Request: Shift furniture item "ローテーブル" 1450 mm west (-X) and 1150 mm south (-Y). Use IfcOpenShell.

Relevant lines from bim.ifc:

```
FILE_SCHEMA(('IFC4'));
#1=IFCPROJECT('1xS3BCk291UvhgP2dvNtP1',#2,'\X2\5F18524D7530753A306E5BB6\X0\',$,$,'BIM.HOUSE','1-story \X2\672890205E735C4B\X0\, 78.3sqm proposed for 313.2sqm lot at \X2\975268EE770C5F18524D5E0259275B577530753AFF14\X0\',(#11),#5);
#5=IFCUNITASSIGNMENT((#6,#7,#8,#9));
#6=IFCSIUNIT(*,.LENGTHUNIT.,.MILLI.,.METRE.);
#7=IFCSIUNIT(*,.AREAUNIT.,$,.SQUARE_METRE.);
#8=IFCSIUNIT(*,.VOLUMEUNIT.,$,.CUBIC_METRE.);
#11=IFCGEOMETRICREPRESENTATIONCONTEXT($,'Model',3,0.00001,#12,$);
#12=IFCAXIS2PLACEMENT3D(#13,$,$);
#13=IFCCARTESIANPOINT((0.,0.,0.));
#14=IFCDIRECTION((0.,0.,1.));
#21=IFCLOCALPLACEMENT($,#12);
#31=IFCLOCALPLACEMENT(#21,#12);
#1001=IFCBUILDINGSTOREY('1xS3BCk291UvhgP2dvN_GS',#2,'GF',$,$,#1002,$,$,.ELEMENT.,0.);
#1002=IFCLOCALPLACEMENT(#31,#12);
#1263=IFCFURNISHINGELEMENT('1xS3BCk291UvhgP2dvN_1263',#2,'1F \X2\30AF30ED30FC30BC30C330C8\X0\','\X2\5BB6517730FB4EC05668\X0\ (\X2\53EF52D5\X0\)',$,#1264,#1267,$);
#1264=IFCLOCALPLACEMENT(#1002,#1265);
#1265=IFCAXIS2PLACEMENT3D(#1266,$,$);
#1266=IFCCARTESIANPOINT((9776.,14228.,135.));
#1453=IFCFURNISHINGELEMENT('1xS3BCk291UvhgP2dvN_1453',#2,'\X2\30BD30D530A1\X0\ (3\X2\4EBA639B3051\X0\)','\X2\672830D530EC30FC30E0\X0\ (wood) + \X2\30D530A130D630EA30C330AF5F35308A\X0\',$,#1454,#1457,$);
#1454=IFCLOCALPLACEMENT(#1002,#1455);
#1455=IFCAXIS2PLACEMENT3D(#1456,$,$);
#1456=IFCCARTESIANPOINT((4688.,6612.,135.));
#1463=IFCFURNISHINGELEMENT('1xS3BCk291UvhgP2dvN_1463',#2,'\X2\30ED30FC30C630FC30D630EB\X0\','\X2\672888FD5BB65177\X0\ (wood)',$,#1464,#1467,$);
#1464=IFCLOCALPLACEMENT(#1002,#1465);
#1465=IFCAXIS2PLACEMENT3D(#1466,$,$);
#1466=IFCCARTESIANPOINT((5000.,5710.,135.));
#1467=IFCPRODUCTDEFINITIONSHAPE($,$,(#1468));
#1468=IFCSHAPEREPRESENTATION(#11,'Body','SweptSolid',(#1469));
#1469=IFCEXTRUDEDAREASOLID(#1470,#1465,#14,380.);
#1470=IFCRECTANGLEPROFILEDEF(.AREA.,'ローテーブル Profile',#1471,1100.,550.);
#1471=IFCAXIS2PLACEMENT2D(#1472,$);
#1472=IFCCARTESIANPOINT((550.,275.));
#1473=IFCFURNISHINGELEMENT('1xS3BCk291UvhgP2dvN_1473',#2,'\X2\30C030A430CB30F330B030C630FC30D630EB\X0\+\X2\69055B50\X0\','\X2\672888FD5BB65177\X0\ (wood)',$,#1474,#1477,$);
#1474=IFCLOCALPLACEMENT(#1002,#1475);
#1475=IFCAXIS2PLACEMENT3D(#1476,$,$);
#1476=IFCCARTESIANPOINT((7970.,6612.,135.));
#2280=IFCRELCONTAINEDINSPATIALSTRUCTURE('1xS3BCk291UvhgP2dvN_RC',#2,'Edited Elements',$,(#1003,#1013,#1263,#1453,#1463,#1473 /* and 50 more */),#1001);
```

```python
import ifcopenshell
import ifcopenshell.api.geometry
import ifcopenshell.util.placement

model = ifcopenshell.open("bim.ifc")

item = model.by_id(1463)
matrix = ifcopenshell.util.placement.get_local_placement(item.ObjectPlacement)
matrix[0, 3] -= 1450.0
matrix[1, 3] -= 1150.0
ifcopenshell.api.geometry.edit_object_placement(model, product=item, matrix=matrix, is_si=False)

print(ifcopenshell.util.placement.get_local_placement(item.ObjectPlacement).round(3) + 0.0)

model.write("bim-out.ifc")
```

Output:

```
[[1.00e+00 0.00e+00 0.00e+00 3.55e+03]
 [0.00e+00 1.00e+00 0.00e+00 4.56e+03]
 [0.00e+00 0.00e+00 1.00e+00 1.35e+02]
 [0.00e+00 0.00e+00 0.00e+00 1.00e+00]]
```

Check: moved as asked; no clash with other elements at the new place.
